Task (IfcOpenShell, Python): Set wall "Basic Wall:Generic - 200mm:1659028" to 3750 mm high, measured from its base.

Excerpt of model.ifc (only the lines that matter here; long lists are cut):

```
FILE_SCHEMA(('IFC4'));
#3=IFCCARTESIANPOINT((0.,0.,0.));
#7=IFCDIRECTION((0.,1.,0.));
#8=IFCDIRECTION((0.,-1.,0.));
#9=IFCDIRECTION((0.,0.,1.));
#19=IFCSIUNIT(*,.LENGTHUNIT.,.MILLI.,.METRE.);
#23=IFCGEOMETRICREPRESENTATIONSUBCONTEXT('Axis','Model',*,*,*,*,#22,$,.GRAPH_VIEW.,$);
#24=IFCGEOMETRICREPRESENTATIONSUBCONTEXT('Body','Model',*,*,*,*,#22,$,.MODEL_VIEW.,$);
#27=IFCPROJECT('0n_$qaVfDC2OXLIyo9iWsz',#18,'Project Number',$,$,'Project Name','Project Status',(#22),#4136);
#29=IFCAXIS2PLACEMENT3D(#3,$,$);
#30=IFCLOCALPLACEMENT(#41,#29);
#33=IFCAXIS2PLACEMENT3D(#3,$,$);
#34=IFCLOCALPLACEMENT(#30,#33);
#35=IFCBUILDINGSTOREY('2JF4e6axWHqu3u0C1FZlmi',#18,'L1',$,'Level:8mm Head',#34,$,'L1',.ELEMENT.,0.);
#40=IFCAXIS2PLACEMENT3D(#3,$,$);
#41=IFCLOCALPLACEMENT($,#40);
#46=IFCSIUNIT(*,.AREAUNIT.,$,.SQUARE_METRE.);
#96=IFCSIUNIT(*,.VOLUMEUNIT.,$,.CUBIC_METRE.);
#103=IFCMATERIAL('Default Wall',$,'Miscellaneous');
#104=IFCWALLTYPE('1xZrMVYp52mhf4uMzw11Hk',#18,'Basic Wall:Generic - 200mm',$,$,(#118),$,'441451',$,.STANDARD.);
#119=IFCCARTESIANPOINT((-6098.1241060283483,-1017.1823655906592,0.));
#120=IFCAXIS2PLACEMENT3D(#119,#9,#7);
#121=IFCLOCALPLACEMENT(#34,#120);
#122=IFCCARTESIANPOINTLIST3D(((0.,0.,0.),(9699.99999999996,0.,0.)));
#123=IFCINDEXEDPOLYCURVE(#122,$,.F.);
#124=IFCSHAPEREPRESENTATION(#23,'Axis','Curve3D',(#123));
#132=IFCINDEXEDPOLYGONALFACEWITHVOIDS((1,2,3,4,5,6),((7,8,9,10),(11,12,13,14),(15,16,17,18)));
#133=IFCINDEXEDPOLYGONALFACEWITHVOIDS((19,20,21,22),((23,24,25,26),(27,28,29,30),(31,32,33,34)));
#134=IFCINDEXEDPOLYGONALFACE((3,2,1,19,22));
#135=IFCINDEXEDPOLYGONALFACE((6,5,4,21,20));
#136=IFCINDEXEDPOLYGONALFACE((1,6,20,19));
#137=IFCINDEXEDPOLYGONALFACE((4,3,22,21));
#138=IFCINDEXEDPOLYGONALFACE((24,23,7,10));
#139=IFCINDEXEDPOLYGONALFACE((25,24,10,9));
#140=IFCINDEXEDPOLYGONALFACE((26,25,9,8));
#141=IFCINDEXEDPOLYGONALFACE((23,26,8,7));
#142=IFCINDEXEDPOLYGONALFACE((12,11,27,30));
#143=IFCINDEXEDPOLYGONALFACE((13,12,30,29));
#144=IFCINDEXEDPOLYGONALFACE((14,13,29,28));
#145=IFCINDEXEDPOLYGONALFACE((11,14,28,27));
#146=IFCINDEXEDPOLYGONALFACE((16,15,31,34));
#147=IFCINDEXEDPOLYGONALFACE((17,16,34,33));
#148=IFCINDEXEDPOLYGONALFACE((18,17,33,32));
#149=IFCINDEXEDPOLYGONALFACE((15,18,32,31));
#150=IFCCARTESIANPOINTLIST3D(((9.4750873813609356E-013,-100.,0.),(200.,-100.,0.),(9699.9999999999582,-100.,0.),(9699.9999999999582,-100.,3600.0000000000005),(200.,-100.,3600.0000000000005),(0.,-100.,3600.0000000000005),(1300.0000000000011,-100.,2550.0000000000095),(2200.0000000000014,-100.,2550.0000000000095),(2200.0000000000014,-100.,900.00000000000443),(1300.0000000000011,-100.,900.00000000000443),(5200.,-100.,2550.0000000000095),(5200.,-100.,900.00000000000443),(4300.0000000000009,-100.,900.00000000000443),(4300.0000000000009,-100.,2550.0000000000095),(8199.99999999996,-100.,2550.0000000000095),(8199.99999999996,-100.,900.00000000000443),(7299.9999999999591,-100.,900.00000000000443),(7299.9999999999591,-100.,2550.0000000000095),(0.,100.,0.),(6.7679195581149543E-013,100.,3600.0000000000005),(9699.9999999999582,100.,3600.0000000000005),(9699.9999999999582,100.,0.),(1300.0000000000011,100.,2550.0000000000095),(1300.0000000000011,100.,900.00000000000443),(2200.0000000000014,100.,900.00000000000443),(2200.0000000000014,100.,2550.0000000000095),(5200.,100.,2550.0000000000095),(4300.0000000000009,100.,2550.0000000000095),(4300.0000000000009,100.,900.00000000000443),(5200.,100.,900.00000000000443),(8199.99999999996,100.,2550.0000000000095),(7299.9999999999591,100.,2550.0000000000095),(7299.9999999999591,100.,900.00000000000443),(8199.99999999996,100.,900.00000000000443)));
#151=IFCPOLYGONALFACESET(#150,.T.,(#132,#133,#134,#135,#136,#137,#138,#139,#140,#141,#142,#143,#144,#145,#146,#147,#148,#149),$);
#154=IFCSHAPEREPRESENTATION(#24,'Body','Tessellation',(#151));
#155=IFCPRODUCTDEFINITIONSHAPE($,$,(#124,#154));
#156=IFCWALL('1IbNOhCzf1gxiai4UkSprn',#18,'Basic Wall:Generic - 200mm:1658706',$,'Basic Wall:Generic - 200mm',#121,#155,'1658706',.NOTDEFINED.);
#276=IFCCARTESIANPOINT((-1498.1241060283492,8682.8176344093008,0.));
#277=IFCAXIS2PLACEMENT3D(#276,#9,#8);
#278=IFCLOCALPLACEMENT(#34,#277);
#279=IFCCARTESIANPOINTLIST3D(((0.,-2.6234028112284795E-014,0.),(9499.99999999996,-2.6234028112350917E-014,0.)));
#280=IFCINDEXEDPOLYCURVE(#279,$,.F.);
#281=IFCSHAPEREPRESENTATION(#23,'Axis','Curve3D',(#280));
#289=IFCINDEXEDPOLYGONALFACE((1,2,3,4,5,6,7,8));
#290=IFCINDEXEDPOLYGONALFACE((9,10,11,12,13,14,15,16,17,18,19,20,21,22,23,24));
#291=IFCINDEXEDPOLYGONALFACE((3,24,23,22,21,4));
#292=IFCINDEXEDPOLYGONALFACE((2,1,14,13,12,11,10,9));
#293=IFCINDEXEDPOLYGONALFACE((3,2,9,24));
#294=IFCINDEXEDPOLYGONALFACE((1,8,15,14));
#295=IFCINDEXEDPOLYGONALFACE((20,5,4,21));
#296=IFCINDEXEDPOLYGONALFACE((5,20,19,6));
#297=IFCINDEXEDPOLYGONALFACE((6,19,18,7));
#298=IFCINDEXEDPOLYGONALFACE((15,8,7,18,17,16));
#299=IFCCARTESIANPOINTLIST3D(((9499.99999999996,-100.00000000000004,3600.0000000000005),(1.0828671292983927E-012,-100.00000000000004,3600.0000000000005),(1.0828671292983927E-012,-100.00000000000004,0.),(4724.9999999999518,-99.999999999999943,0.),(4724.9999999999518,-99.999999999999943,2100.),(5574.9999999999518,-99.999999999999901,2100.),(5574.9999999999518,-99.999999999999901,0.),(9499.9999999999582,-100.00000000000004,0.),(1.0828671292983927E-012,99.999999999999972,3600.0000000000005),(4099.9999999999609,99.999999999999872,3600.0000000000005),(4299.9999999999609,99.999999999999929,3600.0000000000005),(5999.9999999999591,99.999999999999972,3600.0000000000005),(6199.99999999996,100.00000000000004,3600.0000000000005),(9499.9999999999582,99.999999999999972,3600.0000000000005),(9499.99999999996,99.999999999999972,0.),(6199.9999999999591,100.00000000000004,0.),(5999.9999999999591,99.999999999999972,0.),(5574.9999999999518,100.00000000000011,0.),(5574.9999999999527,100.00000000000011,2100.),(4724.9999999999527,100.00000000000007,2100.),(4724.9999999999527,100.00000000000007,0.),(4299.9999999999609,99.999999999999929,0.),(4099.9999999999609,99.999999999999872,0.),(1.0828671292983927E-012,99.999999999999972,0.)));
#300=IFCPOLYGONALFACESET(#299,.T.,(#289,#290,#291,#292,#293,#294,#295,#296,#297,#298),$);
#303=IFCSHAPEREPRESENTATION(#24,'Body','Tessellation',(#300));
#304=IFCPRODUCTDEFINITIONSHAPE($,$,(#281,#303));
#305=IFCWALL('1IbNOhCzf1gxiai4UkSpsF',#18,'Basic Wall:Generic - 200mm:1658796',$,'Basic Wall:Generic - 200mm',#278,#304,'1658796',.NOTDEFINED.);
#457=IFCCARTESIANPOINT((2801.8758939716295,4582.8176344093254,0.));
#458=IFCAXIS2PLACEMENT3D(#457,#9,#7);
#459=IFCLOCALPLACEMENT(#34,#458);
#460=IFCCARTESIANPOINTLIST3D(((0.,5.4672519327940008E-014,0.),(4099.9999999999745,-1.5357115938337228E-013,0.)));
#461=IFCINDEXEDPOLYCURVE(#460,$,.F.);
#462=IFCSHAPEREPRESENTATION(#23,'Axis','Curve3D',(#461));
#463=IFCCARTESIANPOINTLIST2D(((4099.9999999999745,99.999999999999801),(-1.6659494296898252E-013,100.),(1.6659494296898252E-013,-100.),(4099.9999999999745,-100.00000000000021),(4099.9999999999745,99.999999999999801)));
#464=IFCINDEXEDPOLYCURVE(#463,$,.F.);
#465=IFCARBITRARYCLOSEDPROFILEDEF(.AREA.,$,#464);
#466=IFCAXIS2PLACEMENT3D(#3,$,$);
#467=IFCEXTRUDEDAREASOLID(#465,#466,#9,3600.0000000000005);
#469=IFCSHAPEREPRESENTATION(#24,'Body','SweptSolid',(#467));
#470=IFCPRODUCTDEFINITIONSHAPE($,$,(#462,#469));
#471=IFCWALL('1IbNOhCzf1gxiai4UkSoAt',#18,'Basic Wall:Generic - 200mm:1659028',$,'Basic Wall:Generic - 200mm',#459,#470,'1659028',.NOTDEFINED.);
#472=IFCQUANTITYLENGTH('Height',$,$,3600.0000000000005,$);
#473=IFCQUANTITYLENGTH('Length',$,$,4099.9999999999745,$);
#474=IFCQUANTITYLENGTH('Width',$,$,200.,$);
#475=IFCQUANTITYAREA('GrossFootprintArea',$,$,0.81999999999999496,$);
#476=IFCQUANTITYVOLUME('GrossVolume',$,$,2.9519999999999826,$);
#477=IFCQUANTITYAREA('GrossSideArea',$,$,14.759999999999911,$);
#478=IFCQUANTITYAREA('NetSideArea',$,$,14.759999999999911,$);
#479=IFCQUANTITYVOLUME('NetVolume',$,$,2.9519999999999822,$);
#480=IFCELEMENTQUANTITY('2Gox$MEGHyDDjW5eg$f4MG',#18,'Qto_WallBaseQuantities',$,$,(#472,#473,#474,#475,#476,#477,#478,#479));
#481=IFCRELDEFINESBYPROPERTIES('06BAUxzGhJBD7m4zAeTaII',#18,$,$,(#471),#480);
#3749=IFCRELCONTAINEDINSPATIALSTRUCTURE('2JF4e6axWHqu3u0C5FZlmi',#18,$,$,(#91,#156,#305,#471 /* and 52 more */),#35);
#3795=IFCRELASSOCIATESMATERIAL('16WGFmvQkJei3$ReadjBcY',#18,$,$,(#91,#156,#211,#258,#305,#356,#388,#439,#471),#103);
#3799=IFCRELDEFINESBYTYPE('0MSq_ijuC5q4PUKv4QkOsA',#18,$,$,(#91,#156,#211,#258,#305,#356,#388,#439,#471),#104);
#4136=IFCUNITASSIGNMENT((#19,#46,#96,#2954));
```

```python
import ifcopenshell
import ifcopenshell.api.pset
import ifcopenshell.geom
import ifcopenshell.util.element
import ifcopenshell.util.representation
import ifcopenshell.util.shape
import ifcopenshell.util.unit

model = ifcopenshell.open("model.ifc")
unit_scale = ifcopenshell.util.unit.calculate_unit_scale(model)
area_scale = ifcopenshell.util.unit.calculate_unit_scale(model, "AREAUNIT")
volume_scale = ifcopenshell.util.unit.calculate_unit_scale(model, "VOLUMEUNIT")
settings = ifcopenshell.geom.settings()


def volume(element):
    """Net volume in cubic metres, openings subtracted."""
    shape = ifcopenshell.geom.create_shape(settings, element)
    return ifcopenshell.util.shape.get_volume(shape.geometry)


wall = model.by_guid("1IbNOhCzf1gxiai4UkSoAt")
before = volume(wall)

body = ifcopenshell.util.representation.get_representation(wall, "Model", "Body")
solid = body.Items[0]
old_height = solid.Depth
solid.Depth = 3.75 / unit_scale
after = volume(wall)
thickness = 0.2  # wall thickness in metres

# Update the stored height, areas and volumes.
qto = model.by_id(ifcopenshell.util.element.get_pset(wall, "Qto_WallBaseQuantities", should_inherit=False)["id"])
ifcopenshell.api.pset.edit_qto(model, qto=qto, properties={
    "Height": solid.Depth,
    "GrossVolume": ifcopenshell.util.element.get_pset(wall, "Qto_WallBaseQuantities", "GrossVolume") * solid.Depth / old_height,
    "GrossSideArea": ifcopenshell.util.element.get_pset(wall, "Qto_WallBaseQuantities", "GrossSideArea") * solid.Depth / old_height,
    "NetSideArea": after / thickness / area_scale,
    "NetVolume": after / volume_scale,
})

print(f"height {old_height:g} -> {solid.Depth:g}, volume {before:.3f} -> {after:.3f} m3")

model.write("model_v2.ifc")
```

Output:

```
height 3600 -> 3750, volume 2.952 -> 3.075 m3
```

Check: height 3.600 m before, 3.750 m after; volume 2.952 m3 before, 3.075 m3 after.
